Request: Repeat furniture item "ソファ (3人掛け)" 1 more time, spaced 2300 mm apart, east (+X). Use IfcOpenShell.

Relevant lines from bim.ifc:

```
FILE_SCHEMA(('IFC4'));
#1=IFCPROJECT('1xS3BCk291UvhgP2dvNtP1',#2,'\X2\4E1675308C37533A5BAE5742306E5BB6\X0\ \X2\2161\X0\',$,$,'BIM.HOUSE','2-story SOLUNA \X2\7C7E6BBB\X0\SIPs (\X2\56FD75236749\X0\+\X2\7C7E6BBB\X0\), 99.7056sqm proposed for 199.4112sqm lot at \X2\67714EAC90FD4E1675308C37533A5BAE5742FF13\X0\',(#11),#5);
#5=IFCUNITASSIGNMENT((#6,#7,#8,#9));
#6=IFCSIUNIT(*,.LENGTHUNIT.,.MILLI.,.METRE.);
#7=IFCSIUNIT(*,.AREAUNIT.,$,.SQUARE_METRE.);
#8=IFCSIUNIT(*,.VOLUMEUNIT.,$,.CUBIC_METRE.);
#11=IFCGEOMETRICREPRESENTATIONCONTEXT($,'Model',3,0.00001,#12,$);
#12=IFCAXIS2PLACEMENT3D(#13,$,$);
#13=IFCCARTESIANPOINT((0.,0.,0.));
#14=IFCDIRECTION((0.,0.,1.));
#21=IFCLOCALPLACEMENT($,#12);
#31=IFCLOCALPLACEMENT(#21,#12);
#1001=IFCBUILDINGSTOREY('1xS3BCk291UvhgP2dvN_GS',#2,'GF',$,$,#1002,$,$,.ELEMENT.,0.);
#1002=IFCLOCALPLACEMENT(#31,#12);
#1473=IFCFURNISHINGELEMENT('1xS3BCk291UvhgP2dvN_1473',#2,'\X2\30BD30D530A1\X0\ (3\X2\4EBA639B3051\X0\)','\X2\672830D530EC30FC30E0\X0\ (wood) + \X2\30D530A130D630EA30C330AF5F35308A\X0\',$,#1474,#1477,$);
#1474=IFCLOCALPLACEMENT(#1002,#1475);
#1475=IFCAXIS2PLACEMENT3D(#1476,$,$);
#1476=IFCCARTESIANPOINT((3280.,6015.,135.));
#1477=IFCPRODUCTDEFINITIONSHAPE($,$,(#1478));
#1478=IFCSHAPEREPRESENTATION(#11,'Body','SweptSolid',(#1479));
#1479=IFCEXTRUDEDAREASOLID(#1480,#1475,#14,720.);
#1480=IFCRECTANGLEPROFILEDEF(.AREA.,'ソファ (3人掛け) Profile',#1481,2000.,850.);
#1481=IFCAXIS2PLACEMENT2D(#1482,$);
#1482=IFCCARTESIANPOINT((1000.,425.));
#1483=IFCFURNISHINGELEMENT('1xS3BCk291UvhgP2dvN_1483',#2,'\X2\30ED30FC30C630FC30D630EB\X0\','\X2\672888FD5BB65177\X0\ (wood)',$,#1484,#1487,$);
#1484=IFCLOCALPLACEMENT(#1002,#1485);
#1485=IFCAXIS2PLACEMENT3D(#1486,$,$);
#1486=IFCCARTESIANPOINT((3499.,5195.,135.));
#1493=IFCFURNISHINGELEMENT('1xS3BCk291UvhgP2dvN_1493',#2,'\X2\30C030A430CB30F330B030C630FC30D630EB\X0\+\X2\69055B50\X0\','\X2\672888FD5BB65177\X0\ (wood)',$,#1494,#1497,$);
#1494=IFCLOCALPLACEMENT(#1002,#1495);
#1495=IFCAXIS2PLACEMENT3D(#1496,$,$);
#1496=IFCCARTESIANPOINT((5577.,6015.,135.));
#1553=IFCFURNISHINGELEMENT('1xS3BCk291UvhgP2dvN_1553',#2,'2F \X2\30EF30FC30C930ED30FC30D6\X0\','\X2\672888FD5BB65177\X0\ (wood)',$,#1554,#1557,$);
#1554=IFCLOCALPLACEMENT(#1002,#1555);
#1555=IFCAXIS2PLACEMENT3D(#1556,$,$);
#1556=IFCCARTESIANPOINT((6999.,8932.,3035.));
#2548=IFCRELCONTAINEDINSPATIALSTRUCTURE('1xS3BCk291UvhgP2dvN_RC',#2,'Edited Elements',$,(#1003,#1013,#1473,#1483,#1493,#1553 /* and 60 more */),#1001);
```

```python
import numpy as np
import ifcopenshell
import ifcopenshell.api.geometry
import ifcopenshell.api.root
import ifcopenshell.util.element
import ifcopenshell.util.placement
import ifcopenshell.util.unit

model = ifcopenshell.open("bim.ifc")
unit_scale = ifcopenshell.util.unit.calculate_unit_scale(model)


def reuse_history(source, copy):
    """copy_class also copies each property set's owner history, people and application; keep the originals."""
    for rel in copy.IsDefinedBy:
        if rel.is_a("IfcRelDefinesByProperties") and (history := rel.RelatingPropertyDefinition.OwnerHistory):
            rel.RelatingPropertyDefinition.OwnerHistory = source.OwnerHistory
            ifcopenshell.util.element.remove_deep2(model, history)


source = model.by_guid("1xS3BCk291UvhgP2dvN_1473")
base = ifcopenshell.util.placement.get_local_placement(source.ObjectPlacement)
step = np.array([1.0, 0.0, 0.0]) * 2.3 / unit_scale

for i in range(1, 2):
    copy = ifcopenshell.api.root.copy_class(model, product=source)
    copy.Representation = ifcopenshell.util.element.copy_deep(
        model, source.Representation, exclude=["IfcGeometricRepresentationContext", "IfcRepresentationMap"]
    )
    reuse_history(source, copy)
    matrix = base.copy()
    matrix[:3, 3] += i * step
    print("added at", matrix[:3, 3].round(3) + 0.0)
    ifcopenshell.api.geometry.edit_object_placement(model, product=copy, matrix=matrix, is_si=False)

model.write("bim_updated.ifc")
```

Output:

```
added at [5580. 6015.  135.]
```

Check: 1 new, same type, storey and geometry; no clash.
